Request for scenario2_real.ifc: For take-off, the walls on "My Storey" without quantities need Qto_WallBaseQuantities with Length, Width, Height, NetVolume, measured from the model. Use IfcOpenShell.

First a look at what the model holds.

```python
import ifcopenshell
import ifcopenshell.util.element
import ifcopenshell.util.unit

model = ifcopenshell.open("scenario2_real.ifc")
print(model.schema)
for unit_type in ("LENGTHUNIT", "AREAUNIT", "VOLUMEUNIT"):
    print(unit_type, ifcopenshell.util.unit.calculate_unit_scale(model, unit_type))
storey = next(s for s in model.by_type("IfcBuildingStorey") if s.Name == "My Storey")
walls = [e for e in ifcopenshell.util.element.get_decomposition(storey) if e.is_a("IfcWall")]
for e in sorted(walls, key=lambda e: e.id()):
    print(e.id(), e.is_a(), e.Name, list(ifcopenshell.util.element.get_psets(e, qtos_only=True)), sep=" | ")
```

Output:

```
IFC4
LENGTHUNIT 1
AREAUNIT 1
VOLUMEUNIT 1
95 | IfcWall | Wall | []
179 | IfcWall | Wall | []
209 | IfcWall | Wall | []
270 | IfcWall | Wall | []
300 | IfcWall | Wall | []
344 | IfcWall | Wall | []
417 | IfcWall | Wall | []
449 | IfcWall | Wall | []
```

```python
import ifcopenshell
import ifcopenshell.api.pset
import ifcopenshell.geom
import ifcopenshell.util.element
import ifcopenshell.util.shape
import ifcopenshell.util.unit

model = ifcopenshell.open("scenario2_real.ifc")
unit_scale = ifcopenshell.util.unit.calculate_unit_scale(model)
volume_scale = ifcopenshell.util.unit.calculate_unit_scale(model, "VOLUMEUNIT")
settings = ifcopenshell.geom.settings()

storey = next(s for s in model.by_type("IfcBuildingStorey") if s.Name == "My Storey")
walls = [e for e in ifcopenshell.util.element.get_decomposition(storey) if e.is_a("IfcWall")]

for e in sorted(walls, key=lambda e: e.id()):
    if ifcopenshell.util.element.get_psets(e, qtos_only=True, should_inherit=False):
        continue
    # Geometry comes back in metres, in the element's own axes.
    shape = ifcopenshell.geom.create_shape(settings, e)
    values = {
        "Length": ifcopenshell.util.shape.get_x(shape.geometry) / unit_scale,
        "Width": ifcopenshell.util.shape.get_y(shape.geometry) / unit_scale,
        "Height": ifcopenshell.util.shape.get_z(shape.geometry) / unit_scale,
        "NetVolume": ifcopenshell.util.shape.get_volume(shape.geometry) / volume_scale,
    }
    qto = ifcopenshell.api.pset.add_qto(model, product=e, name="Qto_WallBaseQuantities")
    ifcopenshell.api.pset.edit_qto(model, qto=qto, properties=values)
    print(e.id(), {k: round(v, 3) for k, v in values.items()})

model.write("scenario2_real_rev.ifc")
```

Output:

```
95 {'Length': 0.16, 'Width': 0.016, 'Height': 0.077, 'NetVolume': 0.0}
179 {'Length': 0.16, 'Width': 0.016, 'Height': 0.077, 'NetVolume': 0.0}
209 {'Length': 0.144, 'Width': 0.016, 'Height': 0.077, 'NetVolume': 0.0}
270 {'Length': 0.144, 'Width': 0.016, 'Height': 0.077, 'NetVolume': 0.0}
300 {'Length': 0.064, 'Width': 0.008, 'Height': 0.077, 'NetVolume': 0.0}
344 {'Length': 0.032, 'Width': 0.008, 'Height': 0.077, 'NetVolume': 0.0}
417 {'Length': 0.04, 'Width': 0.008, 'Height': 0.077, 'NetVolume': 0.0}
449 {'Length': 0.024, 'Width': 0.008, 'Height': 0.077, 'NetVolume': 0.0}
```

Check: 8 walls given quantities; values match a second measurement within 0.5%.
